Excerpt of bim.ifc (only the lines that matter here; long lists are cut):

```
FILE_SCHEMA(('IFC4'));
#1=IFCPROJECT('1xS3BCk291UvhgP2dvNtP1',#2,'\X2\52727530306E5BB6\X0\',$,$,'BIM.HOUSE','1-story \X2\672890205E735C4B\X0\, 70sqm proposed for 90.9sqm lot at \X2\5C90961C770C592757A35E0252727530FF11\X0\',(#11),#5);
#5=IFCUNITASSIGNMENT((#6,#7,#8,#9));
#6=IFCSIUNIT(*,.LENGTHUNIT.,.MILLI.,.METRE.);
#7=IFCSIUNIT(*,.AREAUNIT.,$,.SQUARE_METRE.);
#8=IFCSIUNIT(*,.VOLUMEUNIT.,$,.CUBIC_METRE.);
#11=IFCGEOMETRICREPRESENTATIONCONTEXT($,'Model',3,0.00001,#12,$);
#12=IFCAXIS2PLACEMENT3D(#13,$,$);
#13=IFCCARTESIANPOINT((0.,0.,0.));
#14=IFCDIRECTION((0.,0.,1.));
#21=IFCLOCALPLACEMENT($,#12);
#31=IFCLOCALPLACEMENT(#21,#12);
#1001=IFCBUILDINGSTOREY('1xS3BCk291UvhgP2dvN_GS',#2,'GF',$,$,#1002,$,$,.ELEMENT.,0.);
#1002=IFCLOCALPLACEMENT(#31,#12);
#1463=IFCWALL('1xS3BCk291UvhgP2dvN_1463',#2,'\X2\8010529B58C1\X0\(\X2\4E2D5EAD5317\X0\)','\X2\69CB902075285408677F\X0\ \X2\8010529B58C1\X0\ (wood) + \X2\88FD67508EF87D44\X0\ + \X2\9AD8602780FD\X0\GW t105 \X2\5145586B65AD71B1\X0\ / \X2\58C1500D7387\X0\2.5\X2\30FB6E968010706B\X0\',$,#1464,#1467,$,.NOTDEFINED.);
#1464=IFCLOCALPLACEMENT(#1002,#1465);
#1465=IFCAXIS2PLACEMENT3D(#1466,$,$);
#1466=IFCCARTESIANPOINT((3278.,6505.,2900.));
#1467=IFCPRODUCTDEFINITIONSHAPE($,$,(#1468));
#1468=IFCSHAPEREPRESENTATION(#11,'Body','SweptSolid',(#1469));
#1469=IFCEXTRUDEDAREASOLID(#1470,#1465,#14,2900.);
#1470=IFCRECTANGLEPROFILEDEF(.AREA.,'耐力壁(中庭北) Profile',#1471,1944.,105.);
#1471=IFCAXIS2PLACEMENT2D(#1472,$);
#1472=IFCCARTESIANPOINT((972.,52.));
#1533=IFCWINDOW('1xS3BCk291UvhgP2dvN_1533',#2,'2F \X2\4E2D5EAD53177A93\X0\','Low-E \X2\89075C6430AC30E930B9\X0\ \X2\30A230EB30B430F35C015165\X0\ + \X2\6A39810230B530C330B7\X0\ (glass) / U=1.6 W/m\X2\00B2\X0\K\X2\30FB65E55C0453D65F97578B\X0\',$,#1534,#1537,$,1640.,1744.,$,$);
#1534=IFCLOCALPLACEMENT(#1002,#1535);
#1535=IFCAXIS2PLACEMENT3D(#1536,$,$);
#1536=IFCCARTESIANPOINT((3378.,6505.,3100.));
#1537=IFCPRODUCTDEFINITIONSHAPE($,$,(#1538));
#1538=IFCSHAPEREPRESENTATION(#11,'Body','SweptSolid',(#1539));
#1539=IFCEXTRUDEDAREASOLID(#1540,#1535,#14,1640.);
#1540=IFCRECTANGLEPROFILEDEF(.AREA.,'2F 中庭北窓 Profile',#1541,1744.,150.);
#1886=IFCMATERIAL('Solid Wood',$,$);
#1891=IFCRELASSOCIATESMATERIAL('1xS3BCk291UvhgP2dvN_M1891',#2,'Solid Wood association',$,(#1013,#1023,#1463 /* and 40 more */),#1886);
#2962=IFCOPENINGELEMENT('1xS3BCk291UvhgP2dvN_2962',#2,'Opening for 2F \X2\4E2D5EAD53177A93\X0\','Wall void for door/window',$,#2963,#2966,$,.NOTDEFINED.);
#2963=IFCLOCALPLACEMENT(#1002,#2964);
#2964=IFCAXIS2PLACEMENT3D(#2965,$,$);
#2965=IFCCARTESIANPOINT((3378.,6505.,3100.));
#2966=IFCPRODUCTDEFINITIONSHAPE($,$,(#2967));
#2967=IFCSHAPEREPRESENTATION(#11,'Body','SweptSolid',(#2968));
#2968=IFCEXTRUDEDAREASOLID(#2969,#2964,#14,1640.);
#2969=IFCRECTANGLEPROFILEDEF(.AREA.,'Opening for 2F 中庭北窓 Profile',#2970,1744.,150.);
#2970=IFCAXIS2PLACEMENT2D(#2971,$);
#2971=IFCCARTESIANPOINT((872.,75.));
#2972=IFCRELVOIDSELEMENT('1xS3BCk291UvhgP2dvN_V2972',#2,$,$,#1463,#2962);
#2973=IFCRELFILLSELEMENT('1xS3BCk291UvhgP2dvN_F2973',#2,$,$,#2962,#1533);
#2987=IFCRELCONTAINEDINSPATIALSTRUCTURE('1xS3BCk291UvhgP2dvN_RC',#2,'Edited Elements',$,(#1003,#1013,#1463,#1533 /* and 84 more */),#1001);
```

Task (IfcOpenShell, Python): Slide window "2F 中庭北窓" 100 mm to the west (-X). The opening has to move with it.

```python
import ifcopenshell
import ifcopenshell.api.geometry
import ifcopenshell.util.placement
import ifcopenshell.util.unit

model = ifcopenshell.open("bim.ifc")
unit_scale = ifcopenshell.util.unit.calculate_unit_scale(model)

window = model.by_guid("1xS3BCk291UvhgP2dvN_1533")
opening = window.FillsVoids[0].RelatingOpeningElement
wall = opening.VoidsElements[0].RelatingBuildingElement

wall_matrix = ifcopenshell.util.placement.get_local_placement(wall.ObjectPlacement)
shift = wall_matrix[:3, 0] * -0.1 / unit_scale
before = ifcopenshell.util.placement.get_local_placement(window.ObjectPlacement)[:3, 3].copy()

# The window is not placed relative to its opening, so move both.
for product in (opening, window):
    matrix = ifcopenshell.util.placement.get_local_placement(product.ObjectPlacement)
    matrix[:3, 3] += shift
    ifcopenshell.api.geometry.edit_object_placement(model, product=product, matrix=matrix, is_si=False)

after = ifcopenshell.util.placement.get_local_placement(window.ObjectPlacement)[:3, 3]
print("window moved by", (after - before).round(3) + 0.0)

model.write("bim_updated.ifc")
```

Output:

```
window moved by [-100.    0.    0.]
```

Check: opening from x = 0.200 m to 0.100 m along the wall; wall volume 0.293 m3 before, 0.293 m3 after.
